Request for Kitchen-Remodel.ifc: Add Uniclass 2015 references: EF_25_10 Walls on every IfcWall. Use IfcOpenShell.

First a look at what the model holds.

```python
import ifcopenshell

model = ifcopenshell.open("Kitchen-Remodel.ifc")
print(model.schema)
print("classifications:", [c.Name for c in model.by_type("IfcClassification")])
for ifc_class in ("IfcDoor", "IfcRoof", "IfcStair", "IfcWall", "IfcWindow"):
    print(ifc_class, len(model.by_type(ifc_class)))
```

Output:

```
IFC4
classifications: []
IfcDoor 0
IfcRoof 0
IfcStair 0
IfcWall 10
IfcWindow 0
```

```python
import ifcopenshell
import ifcopenshell.api.classification

model = ifcopenshell.open("Kitchen-Remodel.ifc")

system = ifcopenshell.api.classification.add_classification(model, classification="Uniclass 2015")

codes = {
    "IfcWall": ("EF_25_10", "Walls"),
}
for ifc_class, (code, name) in codes.items():
    products = model.by_type(ifc_class)
    ifcopenshell.api.classification.add_reference(
        model, products=products, classification=system, identification=code, name=name
    )
    print(code, len(products))

model.write("Kitchen-Remodel_updated.ifc")
```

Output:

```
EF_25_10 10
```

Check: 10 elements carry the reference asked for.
